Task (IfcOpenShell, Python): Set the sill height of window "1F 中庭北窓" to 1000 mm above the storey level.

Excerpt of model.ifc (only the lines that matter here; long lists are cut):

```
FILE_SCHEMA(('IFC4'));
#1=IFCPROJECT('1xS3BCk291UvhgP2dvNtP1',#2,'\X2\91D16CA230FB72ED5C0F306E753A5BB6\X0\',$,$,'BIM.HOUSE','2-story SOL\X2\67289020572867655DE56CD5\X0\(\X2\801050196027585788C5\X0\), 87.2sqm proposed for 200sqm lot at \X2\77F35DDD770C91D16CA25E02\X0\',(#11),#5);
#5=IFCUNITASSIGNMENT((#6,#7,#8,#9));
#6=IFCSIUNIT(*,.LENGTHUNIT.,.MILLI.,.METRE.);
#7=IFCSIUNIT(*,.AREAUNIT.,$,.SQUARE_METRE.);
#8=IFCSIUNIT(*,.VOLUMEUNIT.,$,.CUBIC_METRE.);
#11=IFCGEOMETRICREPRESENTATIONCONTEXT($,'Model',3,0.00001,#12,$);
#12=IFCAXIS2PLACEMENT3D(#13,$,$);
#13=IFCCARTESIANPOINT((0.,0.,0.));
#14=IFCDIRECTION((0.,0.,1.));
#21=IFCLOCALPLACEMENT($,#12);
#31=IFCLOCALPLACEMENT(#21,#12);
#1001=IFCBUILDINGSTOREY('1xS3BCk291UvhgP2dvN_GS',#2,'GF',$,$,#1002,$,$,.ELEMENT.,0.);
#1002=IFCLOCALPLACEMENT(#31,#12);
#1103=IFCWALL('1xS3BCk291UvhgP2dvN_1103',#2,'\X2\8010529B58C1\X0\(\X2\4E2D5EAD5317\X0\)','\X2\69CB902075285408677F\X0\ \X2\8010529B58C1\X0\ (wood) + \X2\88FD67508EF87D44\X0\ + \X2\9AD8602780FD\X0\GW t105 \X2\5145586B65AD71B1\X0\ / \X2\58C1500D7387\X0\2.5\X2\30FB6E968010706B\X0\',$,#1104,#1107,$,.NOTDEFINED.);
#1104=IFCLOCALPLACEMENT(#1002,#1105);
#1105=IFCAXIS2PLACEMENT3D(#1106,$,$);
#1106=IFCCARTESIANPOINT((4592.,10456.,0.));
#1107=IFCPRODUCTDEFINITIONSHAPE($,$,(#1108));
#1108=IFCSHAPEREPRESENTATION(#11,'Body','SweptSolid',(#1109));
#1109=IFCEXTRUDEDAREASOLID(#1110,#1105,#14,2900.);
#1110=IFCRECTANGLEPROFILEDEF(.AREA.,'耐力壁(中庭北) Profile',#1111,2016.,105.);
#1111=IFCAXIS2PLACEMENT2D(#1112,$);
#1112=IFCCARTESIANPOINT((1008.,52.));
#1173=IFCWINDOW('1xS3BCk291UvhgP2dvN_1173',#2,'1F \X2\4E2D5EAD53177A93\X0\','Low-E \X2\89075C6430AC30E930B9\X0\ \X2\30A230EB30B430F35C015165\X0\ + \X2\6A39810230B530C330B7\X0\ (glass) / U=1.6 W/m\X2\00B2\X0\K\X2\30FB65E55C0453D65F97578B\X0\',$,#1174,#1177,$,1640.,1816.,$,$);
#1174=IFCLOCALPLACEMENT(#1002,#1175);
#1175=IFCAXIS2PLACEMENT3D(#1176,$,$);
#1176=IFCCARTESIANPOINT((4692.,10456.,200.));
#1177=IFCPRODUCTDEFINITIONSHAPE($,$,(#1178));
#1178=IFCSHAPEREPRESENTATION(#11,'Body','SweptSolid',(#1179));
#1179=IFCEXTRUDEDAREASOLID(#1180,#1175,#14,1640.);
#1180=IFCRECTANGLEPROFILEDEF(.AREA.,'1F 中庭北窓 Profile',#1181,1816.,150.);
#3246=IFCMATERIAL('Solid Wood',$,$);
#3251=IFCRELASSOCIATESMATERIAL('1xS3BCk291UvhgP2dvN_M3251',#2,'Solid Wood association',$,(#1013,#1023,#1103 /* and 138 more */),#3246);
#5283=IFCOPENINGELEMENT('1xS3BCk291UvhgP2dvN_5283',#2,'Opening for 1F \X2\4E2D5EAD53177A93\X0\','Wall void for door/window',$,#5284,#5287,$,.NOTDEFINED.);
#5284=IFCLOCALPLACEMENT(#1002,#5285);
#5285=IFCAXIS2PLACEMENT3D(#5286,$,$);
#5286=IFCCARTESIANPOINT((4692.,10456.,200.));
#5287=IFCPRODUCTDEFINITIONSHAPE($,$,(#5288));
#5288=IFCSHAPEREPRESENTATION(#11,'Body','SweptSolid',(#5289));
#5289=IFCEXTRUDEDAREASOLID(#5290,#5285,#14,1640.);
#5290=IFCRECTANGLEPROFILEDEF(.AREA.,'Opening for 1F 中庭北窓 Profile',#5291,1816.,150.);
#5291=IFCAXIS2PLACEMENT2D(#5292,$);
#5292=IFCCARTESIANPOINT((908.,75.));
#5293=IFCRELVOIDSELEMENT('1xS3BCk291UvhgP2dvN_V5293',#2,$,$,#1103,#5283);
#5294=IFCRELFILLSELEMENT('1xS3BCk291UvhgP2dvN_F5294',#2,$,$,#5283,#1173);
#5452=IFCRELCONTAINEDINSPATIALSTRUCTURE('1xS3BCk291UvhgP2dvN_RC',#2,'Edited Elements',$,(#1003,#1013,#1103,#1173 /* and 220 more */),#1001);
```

```python
import numpy as np
import ifcopenshell
import ifcopenshell.api.geometry
import ifcopenshell.geom
import ifcopenshell.util.element
import ifcopenshell.util.placement
import ifcopenshell.util.shape
import ifcopenshell.util.unit

model = ifcopenshell.open("model.ifc")
unit_scale = ifcopenshell.util.unit.calculate_unit_scale(model)

window = model.by_guid("1xS3BCk291UvhgP2dvN_1173")
opening = window.FillsVoids[0].RelatingOpeningElement
storey = ifcopenshell.util.element.get_container(window, ifc_class="IfcBuildingStorey")
level = ifcopenshell.util.placement.get_local_placement(storey.ObjectPlacement)[2, 3]

# The opening's origin need not be at the sill, so measure its lowest point.
shape = ifcopenshell.geom.create_shape(ifcopenshell.geom.settings(), opening)
bottom = ifcopenshell.util.shape.get_shape_bottom_elevation(shape, shape.geometry) / unit_scale
dz = level + 1000.0 - bottom

shift = np.array([0.0, 0.0, dz])
# The window is not placed relative to its opening, so move both.
for product in (opening, window):
    matrix = ifcopenshell.util.placement.get_local_placement(product.ObjectPlacement)
    matrix[:3, 3] += shift
    ifcopenshell.api.geometry.edit_object_placement(model, product=product, matrix=matrix, is_si=False)

print(f"moved by {dz * unit_scale:+.3f} m")

model.write("model_v2.ifc")
```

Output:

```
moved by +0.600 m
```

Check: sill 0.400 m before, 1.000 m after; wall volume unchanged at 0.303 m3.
